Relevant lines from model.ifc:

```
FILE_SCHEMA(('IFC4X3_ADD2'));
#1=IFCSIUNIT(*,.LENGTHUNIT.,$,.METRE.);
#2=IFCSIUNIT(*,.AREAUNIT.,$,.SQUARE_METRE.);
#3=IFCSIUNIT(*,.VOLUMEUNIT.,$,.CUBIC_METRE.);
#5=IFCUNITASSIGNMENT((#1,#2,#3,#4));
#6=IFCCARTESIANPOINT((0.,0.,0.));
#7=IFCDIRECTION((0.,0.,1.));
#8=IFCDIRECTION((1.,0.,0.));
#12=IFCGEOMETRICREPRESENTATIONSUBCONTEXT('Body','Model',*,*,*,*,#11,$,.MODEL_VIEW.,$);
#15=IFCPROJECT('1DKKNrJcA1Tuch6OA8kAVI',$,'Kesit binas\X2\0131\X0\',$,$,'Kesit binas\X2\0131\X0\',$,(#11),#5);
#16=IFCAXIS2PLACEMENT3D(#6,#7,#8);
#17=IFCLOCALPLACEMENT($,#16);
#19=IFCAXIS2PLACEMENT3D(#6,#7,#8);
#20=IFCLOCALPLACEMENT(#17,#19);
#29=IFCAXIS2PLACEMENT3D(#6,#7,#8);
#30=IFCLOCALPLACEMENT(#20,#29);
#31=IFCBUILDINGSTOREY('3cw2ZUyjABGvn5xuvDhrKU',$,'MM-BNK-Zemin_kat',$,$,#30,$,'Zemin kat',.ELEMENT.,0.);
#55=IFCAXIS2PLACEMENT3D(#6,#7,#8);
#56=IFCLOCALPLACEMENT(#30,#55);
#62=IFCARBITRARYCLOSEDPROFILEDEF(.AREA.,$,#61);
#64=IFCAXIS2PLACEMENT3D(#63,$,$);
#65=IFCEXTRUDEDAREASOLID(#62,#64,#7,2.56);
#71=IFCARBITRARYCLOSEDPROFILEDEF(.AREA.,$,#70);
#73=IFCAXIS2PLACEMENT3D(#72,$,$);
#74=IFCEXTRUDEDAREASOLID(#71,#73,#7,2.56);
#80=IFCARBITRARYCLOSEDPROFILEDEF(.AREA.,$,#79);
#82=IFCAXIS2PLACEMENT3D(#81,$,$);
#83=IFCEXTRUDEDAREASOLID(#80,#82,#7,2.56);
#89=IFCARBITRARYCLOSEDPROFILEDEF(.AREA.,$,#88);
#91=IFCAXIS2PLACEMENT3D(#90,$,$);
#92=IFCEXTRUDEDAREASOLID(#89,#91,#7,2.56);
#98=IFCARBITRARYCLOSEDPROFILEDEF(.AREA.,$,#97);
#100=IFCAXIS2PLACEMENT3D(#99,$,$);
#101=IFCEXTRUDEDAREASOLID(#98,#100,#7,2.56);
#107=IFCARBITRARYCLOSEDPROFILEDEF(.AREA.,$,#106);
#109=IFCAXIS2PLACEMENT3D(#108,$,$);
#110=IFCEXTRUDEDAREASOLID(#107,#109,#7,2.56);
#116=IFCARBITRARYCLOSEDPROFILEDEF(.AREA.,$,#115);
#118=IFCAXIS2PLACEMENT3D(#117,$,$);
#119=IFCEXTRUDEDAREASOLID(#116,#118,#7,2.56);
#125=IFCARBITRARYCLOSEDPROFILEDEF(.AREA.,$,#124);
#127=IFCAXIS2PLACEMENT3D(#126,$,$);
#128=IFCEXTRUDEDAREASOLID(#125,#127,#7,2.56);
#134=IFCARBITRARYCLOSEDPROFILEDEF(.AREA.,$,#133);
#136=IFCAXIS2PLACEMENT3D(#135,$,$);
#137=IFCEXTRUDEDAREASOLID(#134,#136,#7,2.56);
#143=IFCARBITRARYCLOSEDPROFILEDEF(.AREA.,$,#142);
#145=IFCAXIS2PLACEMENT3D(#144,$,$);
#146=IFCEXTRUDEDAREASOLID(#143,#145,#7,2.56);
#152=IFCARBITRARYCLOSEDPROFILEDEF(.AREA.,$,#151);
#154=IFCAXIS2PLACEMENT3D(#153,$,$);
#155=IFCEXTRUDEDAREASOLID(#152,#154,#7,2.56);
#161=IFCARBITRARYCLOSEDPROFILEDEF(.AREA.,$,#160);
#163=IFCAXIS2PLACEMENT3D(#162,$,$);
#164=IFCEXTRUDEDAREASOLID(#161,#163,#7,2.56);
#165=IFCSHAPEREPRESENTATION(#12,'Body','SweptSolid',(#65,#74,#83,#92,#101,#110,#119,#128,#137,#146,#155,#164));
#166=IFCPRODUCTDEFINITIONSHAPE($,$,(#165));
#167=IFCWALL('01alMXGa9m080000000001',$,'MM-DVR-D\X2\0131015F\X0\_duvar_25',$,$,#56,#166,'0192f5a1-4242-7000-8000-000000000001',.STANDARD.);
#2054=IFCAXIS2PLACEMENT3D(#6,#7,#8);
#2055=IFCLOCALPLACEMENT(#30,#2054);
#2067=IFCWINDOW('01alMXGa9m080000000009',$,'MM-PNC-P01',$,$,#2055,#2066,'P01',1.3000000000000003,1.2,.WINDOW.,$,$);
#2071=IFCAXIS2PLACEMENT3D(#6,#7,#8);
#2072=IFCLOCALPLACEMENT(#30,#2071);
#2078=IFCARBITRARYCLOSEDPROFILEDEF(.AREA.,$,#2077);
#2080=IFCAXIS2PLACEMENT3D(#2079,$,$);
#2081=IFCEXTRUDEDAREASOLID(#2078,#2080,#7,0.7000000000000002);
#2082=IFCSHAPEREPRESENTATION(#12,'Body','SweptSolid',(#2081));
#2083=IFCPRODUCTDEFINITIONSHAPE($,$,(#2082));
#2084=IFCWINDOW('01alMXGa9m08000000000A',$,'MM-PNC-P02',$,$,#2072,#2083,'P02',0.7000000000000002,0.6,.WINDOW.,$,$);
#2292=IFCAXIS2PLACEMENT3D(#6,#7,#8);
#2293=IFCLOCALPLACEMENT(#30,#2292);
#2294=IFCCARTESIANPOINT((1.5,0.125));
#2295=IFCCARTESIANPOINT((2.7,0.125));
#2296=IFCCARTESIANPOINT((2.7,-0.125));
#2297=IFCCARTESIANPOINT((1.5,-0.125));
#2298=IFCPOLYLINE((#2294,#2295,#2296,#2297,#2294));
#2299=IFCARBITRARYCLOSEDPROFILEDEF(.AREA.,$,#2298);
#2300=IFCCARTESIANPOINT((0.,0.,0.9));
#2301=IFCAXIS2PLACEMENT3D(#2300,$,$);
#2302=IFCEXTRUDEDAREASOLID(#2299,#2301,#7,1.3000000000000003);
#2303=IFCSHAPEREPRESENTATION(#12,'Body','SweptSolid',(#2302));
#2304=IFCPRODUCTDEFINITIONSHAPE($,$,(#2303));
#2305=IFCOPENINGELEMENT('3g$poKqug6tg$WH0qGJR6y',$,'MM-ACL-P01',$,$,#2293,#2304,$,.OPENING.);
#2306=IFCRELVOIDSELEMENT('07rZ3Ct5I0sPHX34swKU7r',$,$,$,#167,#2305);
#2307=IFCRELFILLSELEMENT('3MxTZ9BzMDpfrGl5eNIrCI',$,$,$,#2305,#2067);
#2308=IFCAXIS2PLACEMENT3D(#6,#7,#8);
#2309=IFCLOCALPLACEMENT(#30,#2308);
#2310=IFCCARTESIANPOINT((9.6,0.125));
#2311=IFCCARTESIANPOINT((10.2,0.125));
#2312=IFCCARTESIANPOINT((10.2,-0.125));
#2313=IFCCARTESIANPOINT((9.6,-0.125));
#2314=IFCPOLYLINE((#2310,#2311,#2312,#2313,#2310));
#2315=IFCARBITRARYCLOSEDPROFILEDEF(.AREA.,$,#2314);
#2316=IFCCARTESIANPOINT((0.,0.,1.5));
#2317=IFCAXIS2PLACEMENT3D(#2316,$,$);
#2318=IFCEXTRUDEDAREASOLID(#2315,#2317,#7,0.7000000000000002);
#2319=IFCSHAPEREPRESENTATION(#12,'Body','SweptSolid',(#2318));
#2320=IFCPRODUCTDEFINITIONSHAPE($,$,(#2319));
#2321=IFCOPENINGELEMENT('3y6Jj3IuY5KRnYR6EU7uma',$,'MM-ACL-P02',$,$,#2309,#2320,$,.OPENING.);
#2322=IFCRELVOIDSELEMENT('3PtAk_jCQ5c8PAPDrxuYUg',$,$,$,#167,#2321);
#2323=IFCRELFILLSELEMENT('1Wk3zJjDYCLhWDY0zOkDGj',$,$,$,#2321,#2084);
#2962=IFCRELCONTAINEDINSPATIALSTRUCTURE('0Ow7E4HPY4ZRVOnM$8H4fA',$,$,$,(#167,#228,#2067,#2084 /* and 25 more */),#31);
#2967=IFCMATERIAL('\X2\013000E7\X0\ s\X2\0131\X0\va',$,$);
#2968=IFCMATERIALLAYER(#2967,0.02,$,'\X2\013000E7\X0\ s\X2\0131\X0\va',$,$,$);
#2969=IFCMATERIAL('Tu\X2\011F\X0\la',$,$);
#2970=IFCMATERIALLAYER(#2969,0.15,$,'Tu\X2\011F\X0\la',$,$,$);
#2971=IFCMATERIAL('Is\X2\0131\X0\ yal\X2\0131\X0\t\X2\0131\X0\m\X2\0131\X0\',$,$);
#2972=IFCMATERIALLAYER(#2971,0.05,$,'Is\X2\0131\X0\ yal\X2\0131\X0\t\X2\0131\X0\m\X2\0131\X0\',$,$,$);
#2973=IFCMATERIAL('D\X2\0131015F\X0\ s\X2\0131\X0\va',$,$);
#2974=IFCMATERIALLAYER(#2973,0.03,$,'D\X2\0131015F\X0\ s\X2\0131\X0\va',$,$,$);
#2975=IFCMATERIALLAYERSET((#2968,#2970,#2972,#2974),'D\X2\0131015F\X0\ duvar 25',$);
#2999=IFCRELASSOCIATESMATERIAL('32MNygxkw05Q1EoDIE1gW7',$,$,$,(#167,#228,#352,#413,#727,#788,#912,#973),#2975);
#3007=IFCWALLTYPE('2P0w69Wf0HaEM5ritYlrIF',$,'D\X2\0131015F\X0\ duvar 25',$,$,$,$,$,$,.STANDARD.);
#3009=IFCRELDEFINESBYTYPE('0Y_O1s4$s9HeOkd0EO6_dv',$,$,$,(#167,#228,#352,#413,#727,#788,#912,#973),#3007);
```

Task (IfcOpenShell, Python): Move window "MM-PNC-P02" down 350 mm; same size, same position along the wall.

```python
import numpy as np
import ifcopenshell
import ifcopenshell.api.geometry
import ifcopenshell.util.placement
import ifcopenshell.util.unit

model = ifcopenshell.open("model.ifc")
unit_scale = ifcopenshell.util.unit.calculate_unit_scale(model)

window = model.by_guid("01alMXGa9m08000000000A")
opening = window.FillsVoids[0].RelatingOpeningElement
dz = -0.35 / unit_scale

shift = np.array([0.0, 0.0, dz])
# The window is not placed relative to its opening, so move both.
for product in (opening, window):
    matrix = ifcopenshell.util.placement.get_local_placement(product.ObjectPlacement)
    matrix[:3, 3] += shift
    ifcopenshell.api.geometry.edit_object_placement(model, product=product, matrix=matrix, is_si=False)

print(f"moved by {dz * unit_scale:+.3f} m")

model.write("model-out.ifc")
```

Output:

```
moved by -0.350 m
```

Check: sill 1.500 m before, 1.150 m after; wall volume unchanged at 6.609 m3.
